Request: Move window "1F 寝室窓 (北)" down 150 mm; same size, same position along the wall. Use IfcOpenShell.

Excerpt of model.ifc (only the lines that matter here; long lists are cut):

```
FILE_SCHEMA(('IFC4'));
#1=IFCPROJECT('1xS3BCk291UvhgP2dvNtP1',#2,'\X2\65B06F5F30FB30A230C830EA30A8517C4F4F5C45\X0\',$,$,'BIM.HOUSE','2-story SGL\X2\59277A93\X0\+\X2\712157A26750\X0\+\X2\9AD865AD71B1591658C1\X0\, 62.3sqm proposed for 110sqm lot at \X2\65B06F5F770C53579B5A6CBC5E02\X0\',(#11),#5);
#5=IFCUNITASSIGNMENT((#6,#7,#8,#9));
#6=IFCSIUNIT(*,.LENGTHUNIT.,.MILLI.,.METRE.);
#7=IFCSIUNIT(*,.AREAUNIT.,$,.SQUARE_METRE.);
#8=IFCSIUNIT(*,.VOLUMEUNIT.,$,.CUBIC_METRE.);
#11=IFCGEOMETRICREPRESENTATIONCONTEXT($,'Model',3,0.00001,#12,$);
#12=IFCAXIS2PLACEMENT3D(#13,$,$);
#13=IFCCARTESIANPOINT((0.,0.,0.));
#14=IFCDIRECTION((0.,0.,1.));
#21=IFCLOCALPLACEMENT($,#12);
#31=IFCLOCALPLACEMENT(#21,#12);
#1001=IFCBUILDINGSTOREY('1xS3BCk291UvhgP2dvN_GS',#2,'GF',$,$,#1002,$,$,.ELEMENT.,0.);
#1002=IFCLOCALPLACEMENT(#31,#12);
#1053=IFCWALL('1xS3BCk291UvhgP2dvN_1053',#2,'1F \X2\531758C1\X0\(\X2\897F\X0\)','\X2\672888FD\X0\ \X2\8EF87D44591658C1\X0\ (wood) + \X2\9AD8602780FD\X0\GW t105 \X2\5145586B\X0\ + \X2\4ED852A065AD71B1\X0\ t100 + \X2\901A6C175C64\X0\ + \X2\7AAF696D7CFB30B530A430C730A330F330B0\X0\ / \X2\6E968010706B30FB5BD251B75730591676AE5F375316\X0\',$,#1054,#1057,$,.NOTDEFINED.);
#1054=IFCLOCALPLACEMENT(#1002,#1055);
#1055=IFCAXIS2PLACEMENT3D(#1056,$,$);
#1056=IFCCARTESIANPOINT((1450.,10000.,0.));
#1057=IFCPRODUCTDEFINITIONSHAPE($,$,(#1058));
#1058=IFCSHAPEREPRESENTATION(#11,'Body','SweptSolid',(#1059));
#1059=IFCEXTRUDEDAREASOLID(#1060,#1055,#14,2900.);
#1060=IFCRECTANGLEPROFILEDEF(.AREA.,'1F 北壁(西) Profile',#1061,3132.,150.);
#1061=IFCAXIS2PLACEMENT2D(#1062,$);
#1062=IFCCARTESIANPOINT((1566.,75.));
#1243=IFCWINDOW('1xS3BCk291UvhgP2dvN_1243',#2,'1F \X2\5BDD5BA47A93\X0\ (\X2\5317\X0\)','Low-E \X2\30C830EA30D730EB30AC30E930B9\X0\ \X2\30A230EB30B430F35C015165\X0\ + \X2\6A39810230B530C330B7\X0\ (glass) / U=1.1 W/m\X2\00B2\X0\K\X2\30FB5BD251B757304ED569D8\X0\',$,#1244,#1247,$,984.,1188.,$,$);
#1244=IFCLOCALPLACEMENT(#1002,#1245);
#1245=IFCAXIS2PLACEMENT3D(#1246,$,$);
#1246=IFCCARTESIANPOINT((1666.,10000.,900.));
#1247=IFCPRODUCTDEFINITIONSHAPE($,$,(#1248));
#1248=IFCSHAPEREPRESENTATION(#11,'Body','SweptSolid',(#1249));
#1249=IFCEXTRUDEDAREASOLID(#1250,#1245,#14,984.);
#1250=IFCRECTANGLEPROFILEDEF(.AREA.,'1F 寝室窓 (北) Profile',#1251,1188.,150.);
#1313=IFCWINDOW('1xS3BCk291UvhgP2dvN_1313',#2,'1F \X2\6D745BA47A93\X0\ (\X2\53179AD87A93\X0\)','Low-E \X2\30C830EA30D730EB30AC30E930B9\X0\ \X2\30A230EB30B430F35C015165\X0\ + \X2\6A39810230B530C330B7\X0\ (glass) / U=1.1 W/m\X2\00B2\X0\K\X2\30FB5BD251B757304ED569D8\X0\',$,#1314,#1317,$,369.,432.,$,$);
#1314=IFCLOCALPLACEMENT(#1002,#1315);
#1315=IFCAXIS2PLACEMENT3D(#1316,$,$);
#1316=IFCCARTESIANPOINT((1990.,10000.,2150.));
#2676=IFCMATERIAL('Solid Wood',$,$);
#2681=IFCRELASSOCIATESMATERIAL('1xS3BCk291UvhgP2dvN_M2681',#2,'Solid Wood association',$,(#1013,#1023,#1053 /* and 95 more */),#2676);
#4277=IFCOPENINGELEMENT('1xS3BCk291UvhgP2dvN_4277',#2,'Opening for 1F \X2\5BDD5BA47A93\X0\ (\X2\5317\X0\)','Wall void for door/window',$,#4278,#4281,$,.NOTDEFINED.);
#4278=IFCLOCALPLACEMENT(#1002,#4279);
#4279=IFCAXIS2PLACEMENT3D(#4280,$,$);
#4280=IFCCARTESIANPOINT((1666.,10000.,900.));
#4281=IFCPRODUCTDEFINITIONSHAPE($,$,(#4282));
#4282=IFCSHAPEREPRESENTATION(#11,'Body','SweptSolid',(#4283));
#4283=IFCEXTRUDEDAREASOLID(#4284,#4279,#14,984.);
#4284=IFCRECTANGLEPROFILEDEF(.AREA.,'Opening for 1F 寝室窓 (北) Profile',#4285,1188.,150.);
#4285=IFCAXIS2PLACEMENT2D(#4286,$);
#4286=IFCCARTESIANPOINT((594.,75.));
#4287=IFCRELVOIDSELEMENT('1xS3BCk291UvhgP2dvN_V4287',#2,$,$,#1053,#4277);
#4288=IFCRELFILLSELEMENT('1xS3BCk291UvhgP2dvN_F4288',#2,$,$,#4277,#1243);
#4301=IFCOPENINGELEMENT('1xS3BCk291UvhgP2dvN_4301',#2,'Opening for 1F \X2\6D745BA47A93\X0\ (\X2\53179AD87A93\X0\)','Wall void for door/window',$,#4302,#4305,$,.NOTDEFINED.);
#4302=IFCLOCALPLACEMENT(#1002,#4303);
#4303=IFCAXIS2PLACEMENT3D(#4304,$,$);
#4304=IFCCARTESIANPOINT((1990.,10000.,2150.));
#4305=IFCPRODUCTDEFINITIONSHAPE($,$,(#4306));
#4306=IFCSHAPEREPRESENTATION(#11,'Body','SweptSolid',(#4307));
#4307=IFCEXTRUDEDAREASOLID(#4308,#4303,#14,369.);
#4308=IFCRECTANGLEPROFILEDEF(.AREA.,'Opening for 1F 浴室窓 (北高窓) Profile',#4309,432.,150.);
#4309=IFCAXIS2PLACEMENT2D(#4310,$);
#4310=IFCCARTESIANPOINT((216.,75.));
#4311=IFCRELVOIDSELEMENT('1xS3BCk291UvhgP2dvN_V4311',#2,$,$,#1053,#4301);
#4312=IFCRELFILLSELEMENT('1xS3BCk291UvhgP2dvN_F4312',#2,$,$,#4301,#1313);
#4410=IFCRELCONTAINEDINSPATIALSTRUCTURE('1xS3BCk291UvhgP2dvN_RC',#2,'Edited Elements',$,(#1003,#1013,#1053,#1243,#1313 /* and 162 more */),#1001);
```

```python
import numpy as np
import ifcopenshell
import ifcopenshell.api.geometry
import ifcopenshell.util.placement
import ifcopenshell.util.unit

model = ifcopenshell.open("model.ifc")
unit_scale = ifcopenshell.util.unit.calculate_unit_scale(model)

window = model.by_guid("1xS3BCk291UvhgP2dvN_1243")
opening = window.FillsVoids[0].RelatingOpeningElement
dz = -0.15 / unit_scale

shift = np.array([0.0, 0.0, dz])
# The window is not placed relative to its opening, so move both.
for product in (opening, window):
    matrix = ifcopenshell.util.placement.get_local_placement(product.ObjectPlacement)
    matrix[:3, 3] += shift
    ifcopenshell.api.geometry.edit_object_placement(model, product=product, matrix=matrix, is_si=False)

print(f"moved by {dz * unit_scale:+.3f} m")

model.write("model_edited.ifc")
```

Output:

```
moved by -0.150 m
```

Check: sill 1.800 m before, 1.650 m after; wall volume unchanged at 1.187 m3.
